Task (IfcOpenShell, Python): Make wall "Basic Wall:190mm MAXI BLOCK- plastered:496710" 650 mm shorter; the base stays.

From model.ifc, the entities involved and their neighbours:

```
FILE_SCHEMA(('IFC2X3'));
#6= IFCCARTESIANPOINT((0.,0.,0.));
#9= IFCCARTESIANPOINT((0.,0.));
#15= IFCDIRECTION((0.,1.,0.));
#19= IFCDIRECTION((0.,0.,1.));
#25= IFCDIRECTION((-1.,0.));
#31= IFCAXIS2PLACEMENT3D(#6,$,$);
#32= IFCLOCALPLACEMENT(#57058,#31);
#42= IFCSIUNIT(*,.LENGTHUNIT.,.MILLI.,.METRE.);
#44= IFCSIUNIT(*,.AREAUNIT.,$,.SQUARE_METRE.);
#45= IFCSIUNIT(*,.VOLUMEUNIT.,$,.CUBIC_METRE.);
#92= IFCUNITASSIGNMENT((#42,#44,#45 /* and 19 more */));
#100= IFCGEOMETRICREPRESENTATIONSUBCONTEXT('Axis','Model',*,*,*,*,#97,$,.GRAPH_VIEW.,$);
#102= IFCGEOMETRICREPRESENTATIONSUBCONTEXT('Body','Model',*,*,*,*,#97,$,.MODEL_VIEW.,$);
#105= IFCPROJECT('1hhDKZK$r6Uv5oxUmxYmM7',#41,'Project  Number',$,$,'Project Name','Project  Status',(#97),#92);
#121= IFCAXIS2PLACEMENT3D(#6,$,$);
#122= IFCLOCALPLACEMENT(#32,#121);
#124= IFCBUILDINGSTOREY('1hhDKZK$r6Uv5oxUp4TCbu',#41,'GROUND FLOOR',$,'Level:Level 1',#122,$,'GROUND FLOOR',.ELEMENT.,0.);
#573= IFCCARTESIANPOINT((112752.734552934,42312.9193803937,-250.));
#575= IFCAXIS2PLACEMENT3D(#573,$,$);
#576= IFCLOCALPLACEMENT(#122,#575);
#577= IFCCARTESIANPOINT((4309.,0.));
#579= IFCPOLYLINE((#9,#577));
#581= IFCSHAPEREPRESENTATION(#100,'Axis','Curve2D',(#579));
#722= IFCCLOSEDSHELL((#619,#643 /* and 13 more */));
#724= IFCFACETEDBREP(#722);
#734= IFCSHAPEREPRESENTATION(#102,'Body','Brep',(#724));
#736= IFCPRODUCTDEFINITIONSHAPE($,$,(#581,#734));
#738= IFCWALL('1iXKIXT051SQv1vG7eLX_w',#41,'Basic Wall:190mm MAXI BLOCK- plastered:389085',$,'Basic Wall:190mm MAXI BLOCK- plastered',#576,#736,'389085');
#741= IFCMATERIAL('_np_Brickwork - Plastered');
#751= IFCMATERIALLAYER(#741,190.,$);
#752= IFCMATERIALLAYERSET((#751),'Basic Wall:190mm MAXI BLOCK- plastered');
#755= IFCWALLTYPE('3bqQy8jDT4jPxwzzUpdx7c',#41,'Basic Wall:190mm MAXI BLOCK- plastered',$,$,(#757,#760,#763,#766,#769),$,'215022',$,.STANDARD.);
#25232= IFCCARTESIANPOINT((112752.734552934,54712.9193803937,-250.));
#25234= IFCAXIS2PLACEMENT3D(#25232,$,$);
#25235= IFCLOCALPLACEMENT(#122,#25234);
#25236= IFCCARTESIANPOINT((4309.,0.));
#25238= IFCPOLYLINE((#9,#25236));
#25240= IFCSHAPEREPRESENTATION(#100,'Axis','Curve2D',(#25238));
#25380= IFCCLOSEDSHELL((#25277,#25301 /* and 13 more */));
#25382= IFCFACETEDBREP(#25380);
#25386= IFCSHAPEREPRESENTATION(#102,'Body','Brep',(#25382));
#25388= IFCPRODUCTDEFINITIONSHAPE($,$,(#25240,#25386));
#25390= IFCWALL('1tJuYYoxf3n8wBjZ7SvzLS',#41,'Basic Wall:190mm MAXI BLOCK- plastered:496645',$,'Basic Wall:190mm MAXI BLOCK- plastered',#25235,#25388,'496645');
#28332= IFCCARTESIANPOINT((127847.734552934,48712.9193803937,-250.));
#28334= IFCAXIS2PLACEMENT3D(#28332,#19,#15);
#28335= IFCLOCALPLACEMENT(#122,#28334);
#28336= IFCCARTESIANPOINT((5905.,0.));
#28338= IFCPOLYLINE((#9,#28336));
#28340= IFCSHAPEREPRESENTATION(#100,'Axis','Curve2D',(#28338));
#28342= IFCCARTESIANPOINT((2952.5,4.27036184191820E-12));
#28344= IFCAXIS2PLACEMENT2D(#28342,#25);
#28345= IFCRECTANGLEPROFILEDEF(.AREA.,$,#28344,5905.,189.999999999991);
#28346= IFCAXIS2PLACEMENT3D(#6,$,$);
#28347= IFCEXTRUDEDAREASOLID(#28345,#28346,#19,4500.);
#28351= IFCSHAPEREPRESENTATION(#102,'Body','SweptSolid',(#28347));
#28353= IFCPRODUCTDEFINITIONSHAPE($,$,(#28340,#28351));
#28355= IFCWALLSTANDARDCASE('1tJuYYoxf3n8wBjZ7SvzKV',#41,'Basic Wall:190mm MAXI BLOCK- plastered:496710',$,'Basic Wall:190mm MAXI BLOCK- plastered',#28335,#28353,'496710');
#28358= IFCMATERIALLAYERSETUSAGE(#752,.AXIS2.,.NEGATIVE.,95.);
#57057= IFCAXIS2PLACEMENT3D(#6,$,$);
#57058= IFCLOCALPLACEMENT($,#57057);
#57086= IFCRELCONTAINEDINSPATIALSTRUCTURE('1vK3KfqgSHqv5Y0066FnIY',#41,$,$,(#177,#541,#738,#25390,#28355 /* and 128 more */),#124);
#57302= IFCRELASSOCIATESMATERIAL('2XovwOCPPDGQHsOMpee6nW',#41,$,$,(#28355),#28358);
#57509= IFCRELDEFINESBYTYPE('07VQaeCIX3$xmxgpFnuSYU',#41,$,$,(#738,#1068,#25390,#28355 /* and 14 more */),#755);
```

```python
import ifcopenshell
import ifcopenshell.geom
import ifcopenshell.util.representation
import ifcopenshell.util.shape

model = ifcopenshell.open("model.ifc")
settings = ifcopenshell.geom.settings()


def volume(element):
    """Net volume in cubic metres, openings subtracted."""
    shape = ifcopenshell.geom.create_shape(settings, element)
    return ifcopenshell.util.shape.get_volume(shape.geometry)


wall = model.by_id(28355)
before = volume(wall)

body = ifcopenshell.util.representation.get_representation(wall, "Model", "Body")
solid = body.Items[0]
old_height = solid.Depth
solid.Depth -= 650.0
after = volume(wall)

print(f"height {old_height:g} -> {solid.Depth:g}, volume {before:.3f} -> {after:.3f} m3")

model.write("model_rev.ifc")
```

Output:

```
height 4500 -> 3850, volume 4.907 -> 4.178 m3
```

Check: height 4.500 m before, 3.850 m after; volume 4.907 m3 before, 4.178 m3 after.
